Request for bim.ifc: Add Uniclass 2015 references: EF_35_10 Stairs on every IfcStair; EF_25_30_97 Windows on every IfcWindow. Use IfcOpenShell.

First a look at what the model holds.

```python
import ifcopenshell

model = ifcopenshell.open("bim.ifc")
print(model.schema)
print("classifications:", [c.Name for c in model.by_type("IfcClassification")])
for ifc_class in ("IfcDoor", "IfcRoof", "IfcStair", "IfcWall", "IfcWindow"):
    print(ifc_class, len(model.by_type(ifc_class)))
```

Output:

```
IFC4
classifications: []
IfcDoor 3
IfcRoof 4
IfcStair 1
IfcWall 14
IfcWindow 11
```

```python
import ifcopenshell
import ifcopenshell.api.classification

model = ifcopenshell.open("bim.ifc")

system = ifcopenshell.api.classification.add_classification(model, classification="Uniclass 2015")

codes = {
    "IfcStair": ("EF_35_10", "Stairs"),
    "IfcWindow": ("EF_25_30_97", "Windows"),
}
for ifc_class, (code, name) in codes.items():
    products = model.by_type(ifc_class)
    ifcopenshell.api.classification.add_reference(
        model, products=products, classification=system, identification=code, name=name
    )
    print(code, len(products))

model.write("bim_rev.ifc")
```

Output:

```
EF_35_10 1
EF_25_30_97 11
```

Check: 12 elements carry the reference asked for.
